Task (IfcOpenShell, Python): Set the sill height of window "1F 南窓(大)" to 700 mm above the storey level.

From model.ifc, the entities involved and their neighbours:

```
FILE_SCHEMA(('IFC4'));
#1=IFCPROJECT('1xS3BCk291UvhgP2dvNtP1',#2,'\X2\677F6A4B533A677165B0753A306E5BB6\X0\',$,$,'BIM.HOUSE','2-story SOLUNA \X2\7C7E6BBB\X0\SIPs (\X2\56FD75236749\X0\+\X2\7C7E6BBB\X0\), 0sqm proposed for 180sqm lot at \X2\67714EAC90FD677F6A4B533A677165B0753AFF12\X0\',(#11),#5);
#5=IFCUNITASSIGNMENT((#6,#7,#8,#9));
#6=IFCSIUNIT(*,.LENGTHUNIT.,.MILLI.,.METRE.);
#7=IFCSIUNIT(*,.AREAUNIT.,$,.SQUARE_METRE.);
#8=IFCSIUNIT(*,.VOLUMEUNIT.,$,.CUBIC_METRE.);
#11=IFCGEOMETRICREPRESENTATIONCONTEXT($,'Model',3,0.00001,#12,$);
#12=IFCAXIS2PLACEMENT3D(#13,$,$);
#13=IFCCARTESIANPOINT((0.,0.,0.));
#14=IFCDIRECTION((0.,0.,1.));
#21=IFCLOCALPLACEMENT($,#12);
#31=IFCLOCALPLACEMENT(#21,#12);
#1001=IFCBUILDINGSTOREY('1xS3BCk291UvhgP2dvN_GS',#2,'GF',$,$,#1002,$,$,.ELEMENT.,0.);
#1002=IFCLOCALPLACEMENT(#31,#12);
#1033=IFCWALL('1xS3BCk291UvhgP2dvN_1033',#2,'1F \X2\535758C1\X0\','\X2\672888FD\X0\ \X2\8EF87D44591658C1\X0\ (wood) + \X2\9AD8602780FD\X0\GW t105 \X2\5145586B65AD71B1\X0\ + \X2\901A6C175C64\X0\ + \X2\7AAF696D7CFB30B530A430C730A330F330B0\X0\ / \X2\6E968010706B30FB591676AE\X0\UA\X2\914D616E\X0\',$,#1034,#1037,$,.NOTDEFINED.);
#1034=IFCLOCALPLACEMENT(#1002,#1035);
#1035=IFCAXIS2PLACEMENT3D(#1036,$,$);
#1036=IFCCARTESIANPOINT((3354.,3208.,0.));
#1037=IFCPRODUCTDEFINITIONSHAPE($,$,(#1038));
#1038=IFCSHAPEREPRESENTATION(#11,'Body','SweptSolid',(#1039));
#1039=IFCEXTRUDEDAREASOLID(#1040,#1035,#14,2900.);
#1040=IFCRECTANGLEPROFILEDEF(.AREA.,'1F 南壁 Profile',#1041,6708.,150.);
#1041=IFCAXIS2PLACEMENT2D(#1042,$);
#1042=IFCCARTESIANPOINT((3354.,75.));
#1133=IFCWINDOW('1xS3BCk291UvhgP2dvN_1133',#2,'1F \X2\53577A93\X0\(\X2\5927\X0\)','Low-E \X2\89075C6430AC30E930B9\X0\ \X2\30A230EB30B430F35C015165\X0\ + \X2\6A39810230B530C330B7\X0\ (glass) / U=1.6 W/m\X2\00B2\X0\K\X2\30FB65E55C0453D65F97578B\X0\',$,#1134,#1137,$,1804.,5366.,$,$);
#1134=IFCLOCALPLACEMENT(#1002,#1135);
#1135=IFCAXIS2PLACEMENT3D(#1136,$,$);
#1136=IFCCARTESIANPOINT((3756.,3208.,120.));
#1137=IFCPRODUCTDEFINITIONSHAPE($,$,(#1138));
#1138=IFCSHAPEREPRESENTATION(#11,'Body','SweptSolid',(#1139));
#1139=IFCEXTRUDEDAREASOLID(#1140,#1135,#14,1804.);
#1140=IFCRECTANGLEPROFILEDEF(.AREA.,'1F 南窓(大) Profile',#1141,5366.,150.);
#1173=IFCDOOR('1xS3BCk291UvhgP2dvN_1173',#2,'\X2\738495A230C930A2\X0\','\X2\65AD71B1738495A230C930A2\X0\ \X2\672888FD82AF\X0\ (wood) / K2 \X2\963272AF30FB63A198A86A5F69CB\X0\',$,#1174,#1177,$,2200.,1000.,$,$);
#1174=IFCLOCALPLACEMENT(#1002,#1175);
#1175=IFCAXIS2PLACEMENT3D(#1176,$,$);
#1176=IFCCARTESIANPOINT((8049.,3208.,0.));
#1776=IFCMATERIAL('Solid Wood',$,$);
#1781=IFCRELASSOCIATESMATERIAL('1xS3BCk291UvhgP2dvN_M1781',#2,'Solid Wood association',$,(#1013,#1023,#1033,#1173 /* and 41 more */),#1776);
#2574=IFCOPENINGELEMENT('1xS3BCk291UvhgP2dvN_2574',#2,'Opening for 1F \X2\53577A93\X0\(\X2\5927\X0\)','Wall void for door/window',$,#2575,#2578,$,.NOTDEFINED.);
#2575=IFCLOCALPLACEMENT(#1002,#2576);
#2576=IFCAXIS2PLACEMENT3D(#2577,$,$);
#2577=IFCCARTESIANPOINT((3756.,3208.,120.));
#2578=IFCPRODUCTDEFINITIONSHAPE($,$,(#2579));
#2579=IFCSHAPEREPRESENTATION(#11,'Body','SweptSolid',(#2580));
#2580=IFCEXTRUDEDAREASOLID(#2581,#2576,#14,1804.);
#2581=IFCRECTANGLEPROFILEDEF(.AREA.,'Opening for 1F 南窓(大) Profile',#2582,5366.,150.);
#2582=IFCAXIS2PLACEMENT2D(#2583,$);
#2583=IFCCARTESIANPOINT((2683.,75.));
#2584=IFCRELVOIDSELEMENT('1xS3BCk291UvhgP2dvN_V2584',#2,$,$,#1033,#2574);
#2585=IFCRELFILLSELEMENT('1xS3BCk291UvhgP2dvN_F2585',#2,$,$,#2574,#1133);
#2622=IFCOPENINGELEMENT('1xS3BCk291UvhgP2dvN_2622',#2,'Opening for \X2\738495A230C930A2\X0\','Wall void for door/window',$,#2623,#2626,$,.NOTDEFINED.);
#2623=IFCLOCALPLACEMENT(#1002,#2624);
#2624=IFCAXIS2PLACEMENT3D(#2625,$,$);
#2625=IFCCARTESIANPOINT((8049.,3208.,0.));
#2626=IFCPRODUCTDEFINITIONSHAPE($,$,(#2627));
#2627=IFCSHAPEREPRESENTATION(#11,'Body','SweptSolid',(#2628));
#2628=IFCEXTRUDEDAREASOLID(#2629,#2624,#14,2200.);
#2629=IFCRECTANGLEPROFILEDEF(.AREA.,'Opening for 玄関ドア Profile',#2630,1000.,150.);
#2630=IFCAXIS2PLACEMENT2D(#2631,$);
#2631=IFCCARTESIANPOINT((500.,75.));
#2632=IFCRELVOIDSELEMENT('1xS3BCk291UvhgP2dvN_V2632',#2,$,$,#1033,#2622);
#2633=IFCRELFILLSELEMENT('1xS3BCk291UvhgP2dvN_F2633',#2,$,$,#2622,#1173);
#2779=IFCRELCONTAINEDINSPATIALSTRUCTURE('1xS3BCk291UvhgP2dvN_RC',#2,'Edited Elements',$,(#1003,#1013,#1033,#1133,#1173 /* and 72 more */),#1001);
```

```python
import numpy as np
import ifcopenshell
import ifcopenshell.api.geometry
import ifcopenshell.geom
import ifcopenshell.util.element
import ifcopenshell.util.placement
import ifcopenshell.util.shape
import ifcopenshell.util.unit

model = ifcopenshell.open("model.ifc")
unit_scale = ifcopenshell.util.unit.calculate_unit_scale(model)

window = model.by_guid("1xS3BCk291UvhgP2dvN_1133")
opening = window.FillsVoids[0].RelatingOpeningElement
storey = ifcopenshell.util.element.get_container(window, ifc_class="IfcBuildingStorey")
level = ifcopenshell.util.placement.get_local_placement(storey.ObjectPlacement)[2, 3]

# The opening's origin need not be at the sill, so measure its lowest point.
shape = ifcopenshell.geom.create_shape(ifcopenshell.geom.settings(), opening)
bottom = ifcopenshell.util.shape.get_shape_bottom_elevation(shape, shape.geometry) / unit_scale
dz = level + 700.0 - bottom

shift = np.array([0.0, 0.0, dz])
# The window is not placed relative to its opening, so move both.
for product in (opening, window):
    matrix = ifcopenshell.util.placement.get_local_placement(product.ObjectPlacement)
    matrix[:3, 3] += shift
    ifcopenshell.api.geometry.edit_object_placement(model, product=product, matrix=matrix, is_si=False)

print(f"moved by {dz * unit_scale:+.3f} m")

model.write("model-out.ifc")
```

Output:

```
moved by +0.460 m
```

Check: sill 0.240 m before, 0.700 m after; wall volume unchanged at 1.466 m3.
